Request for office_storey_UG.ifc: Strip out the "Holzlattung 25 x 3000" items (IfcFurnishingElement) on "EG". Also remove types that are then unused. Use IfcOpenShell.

First a look at what the model holds.

```python
import ifcopenshell
import ifcopenshell.util.element

model = ifcopenshell.open("office_storey_UG.ifc")
print(model.schema)
storey = next(s for s in model.by_type("IfcBuildingStorey") if s.Name == "EG")
furniture = [e for e in ifcopenshell.util.element.get_decomposition(storey) if e.is_a("IfcFurnishingElement")]
seen = {}
for e in furniture:
    element_type = ifcopenshell.util.element.get_type(e)
    name = element_type.Name if element_type not in (None, e) else None
    seen[name] = seen.get(name, 0) + 1
for name, count in sorted(seen.items(), key=str):
    print(count, "x", name)
```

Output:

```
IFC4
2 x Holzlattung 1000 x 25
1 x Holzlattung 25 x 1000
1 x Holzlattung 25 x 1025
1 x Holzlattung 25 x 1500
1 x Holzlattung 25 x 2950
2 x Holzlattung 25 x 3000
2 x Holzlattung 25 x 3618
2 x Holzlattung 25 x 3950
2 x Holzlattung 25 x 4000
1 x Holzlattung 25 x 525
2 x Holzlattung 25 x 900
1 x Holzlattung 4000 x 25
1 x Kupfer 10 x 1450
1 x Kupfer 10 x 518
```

```python
import ifcopenshell
import ifcopenshell.api.root
import ifcopenshell.util.element

model = ifcopenshell.open("office_storey_UG.ifc")

storey = next(s for s in model.by_type("IfcBuildingStorey") if s.Name == "EG")
furniture = [e for e in ifcopenshell.util.element.get_decomposition(storey) if e.is_a("IfcFurnishingElement")]
targets = [e for e in furniture if (t := ifcopenshell.util.element.get_type(e)) not in (None, e) and t.Name == "Holzlattung 25 x 3000"]
types = {ifcopenshell.util.element.get_type(e) for e in targets} - {None, *targets}

for e in targets:
    ifcopenshell.api.root.remove_product(model, product=e)
print(len(targets), "removed")

unused = [t for t in types if not ifcopenshell.util.element.get_types(t)]
for t in unused:
    ifcopenshell.api.root.remove_product(model, product=t)
print(len(unused), "unused types removed")

model.write("office_storey_UG_updated.ifc")
```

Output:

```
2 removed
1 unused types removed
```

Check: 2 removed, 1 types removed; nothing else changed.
